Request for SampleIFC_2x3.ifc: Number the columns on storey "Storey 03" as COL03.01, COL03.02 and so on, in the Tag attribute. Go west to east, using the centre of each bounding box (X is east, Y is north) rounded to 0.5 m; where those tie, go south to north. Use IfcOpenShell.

First a look at what the model holds.

```python
import ifcopenshell
import ifcopenshell.util.element
import ifcopenshell.util.placement

model = ifcopenshell.open("SampleIFC_2x3.ifc")
print(model.schema)
storey = next(s for s in model.by_type("IfcBuildingStorey") if s.Name == "Storey 03")
columns = [e for e in ifcopenshell.util.element.get_decomposition(storey) if e.is_a("IfcColumn")]
for e in sorted(columns, key=lambda e: e.id()):
    origin = ifcopenshell.util.placement.get_local_placement(e.ObjectPlacement)[:3, 3]
    print(e.id(), e.Tag, e.Name, origin.round(2) + 0.0, sep=" | ")
```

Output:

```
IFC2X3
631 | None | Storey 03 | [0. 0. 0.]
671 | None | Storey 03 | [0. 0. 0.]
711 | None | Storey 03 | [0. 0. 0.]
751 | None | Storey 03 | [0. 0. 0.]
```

```python
import ifcopenshell
import ifcopenshell.geom
import ifcopenshell.util.element
import ifcopenshell.util.shape

model = ifcopenshell.open("SampleIFC_2x3.ifc")
settings = ifcopenshell.geom.settings()
settings.set("use-world-coords", True)


def centre(element):
    shape = ifcopenshell.geom.create_shape(settings, element)
    return ifcopenshell.util.shape.get_bbox_centroid(shape.geometry)


storey = next(s for s in model.by_type("IfcBuildingStorey") if s.Name == "Storey 03")
columns = [e for e in ifcopenshell.util.element.get_decomposition(storey) if e.is_a("IfcColumn")]

# Insertion points can sit at a corner or the storey origin, so sort by the geometry (in metres).
centres = {e: centre(e) for e in columns}
columns.sort(key=lambda e: (round(centres[e][0] / 0.5), centres[e][1]))

for i, e in enumerate(columns, start=1):
    number = f"COL03.{i:02d}"
    e.Tag = number
    print(e.id(), number)

model.write("SampleIFC_2x3-out.ifc")
```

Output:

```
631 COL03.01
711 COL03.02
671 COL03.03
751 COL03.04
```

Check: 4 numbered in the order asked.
